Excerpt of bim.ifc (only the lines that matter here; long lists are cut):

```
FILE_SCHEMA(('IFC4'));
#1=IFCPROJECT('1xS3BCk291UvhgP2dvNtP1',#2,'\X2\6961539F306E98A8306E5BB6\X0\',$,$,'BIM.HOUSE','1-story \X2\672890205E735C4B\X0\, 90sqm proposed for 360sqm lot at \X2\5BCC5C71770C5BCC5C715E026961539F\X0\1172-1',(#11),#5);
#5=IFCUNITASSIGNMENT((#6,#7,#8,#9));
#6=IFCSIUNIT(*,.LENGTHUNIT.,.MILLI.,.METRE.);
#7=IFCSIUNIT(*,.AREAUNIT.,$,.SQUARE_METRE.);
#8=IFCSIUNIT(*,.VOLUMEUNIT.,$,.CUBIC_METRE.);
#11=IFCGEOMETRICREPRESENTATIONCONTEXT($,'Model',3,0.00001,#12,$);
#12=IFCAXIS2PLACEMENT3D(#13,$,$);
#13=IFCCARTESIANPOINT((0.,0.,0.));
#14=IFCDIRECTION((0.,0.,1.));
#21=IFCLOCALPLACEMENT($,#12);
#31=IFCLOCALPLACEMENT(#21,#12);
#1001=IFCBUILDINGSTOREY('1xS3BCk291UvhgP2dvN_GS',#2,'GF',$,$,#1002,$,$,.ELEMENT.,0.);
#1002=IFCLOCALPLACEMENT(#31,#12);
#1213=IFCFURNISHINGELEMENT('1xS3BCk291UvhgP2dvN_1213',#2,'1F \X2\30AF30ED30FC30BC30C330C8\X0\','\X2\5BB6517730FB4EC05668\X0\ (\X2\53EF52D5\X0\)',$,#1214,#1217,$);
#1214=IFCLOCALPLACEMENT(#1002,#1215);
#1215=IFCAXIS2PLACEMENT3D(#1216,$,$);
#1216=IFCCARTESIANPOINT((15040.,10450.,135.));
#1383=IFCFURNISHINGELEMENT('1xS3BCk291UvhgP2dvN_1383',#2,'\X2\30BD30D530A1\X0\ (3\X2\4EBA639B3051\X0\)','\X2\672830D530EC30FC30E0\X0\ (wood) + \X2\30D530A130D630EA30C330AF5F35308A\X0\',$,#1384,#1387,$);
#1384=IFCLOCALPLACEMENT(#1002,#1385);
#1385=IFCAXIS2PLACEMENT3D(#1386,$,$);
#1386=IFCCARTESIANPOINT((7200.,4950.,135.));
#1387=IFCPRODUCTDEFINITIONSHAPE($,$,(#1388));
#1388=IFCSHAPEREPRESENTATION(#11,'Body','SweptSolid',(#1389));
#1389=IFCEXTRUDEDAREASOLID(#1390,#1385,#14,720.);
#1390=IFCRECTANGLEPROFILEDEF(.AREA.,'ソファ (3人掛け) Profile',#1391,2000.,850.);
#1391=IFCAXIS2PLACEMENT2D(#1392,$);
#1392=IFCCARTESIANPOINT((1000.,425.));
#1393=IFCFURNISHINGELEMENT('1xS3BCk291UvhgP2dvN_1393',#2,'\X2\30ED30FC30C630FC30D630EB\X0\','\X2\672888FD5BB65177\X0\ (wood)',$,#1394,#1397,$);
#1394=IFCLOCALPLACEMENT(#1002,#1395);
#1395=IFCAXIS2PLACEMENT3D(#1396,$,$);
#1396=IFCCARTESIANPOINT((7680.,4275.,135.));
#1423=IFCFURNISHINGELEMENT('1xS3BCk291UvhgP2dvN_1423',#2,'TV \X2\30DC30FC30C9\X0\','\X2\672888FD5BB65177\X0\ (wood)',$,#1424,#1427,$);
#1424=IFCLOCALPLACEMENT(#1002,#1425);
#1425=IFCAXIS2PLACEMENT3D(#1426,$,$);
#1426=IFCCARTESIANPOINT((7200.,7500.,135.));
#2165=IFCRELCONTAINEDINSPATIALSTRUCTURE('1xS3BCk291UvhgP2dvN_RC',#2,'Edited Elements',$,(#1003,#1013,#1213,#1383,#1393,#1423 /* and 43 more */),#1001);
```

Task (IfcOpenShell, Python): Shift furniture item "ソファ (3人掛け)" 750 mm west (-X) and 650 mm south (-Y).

```python
import ifcopenshell
import ifcopenshell.api.geometry
import ifcopenshell.util.placement
import ifcopenshell.util.unit

model = ifcopenshell.open("bim.ifc")
unit_scale = ifcopenshell.util.unit.calculate_unit_scale(model)

item = model.by_id(1383)
matrix = ifcopenshell.util.placement.get_local_placement(item.ObjectPlacement)
matrix[0, 3] -= 0.75 / unit_scale
matrix[1, 3] -= 0.65 / unit_scale
ifcopenshell.api.geometry.edit_object_placement(model, product=item, matrix=matrix, is_si=False)

print(ifcopenshell.util.placement.get_local_placement(item.ObjectPlacement).round(3) + 0.0)

model.write("bim_v2.ifc")
```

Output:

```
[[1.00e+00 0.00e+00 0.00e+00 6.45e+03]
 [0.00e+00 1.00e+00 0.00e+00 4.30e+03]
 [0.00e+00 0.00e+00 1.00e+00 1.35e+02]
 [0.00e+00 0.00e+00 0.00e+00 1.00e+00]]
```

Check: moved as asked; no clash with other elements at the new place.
